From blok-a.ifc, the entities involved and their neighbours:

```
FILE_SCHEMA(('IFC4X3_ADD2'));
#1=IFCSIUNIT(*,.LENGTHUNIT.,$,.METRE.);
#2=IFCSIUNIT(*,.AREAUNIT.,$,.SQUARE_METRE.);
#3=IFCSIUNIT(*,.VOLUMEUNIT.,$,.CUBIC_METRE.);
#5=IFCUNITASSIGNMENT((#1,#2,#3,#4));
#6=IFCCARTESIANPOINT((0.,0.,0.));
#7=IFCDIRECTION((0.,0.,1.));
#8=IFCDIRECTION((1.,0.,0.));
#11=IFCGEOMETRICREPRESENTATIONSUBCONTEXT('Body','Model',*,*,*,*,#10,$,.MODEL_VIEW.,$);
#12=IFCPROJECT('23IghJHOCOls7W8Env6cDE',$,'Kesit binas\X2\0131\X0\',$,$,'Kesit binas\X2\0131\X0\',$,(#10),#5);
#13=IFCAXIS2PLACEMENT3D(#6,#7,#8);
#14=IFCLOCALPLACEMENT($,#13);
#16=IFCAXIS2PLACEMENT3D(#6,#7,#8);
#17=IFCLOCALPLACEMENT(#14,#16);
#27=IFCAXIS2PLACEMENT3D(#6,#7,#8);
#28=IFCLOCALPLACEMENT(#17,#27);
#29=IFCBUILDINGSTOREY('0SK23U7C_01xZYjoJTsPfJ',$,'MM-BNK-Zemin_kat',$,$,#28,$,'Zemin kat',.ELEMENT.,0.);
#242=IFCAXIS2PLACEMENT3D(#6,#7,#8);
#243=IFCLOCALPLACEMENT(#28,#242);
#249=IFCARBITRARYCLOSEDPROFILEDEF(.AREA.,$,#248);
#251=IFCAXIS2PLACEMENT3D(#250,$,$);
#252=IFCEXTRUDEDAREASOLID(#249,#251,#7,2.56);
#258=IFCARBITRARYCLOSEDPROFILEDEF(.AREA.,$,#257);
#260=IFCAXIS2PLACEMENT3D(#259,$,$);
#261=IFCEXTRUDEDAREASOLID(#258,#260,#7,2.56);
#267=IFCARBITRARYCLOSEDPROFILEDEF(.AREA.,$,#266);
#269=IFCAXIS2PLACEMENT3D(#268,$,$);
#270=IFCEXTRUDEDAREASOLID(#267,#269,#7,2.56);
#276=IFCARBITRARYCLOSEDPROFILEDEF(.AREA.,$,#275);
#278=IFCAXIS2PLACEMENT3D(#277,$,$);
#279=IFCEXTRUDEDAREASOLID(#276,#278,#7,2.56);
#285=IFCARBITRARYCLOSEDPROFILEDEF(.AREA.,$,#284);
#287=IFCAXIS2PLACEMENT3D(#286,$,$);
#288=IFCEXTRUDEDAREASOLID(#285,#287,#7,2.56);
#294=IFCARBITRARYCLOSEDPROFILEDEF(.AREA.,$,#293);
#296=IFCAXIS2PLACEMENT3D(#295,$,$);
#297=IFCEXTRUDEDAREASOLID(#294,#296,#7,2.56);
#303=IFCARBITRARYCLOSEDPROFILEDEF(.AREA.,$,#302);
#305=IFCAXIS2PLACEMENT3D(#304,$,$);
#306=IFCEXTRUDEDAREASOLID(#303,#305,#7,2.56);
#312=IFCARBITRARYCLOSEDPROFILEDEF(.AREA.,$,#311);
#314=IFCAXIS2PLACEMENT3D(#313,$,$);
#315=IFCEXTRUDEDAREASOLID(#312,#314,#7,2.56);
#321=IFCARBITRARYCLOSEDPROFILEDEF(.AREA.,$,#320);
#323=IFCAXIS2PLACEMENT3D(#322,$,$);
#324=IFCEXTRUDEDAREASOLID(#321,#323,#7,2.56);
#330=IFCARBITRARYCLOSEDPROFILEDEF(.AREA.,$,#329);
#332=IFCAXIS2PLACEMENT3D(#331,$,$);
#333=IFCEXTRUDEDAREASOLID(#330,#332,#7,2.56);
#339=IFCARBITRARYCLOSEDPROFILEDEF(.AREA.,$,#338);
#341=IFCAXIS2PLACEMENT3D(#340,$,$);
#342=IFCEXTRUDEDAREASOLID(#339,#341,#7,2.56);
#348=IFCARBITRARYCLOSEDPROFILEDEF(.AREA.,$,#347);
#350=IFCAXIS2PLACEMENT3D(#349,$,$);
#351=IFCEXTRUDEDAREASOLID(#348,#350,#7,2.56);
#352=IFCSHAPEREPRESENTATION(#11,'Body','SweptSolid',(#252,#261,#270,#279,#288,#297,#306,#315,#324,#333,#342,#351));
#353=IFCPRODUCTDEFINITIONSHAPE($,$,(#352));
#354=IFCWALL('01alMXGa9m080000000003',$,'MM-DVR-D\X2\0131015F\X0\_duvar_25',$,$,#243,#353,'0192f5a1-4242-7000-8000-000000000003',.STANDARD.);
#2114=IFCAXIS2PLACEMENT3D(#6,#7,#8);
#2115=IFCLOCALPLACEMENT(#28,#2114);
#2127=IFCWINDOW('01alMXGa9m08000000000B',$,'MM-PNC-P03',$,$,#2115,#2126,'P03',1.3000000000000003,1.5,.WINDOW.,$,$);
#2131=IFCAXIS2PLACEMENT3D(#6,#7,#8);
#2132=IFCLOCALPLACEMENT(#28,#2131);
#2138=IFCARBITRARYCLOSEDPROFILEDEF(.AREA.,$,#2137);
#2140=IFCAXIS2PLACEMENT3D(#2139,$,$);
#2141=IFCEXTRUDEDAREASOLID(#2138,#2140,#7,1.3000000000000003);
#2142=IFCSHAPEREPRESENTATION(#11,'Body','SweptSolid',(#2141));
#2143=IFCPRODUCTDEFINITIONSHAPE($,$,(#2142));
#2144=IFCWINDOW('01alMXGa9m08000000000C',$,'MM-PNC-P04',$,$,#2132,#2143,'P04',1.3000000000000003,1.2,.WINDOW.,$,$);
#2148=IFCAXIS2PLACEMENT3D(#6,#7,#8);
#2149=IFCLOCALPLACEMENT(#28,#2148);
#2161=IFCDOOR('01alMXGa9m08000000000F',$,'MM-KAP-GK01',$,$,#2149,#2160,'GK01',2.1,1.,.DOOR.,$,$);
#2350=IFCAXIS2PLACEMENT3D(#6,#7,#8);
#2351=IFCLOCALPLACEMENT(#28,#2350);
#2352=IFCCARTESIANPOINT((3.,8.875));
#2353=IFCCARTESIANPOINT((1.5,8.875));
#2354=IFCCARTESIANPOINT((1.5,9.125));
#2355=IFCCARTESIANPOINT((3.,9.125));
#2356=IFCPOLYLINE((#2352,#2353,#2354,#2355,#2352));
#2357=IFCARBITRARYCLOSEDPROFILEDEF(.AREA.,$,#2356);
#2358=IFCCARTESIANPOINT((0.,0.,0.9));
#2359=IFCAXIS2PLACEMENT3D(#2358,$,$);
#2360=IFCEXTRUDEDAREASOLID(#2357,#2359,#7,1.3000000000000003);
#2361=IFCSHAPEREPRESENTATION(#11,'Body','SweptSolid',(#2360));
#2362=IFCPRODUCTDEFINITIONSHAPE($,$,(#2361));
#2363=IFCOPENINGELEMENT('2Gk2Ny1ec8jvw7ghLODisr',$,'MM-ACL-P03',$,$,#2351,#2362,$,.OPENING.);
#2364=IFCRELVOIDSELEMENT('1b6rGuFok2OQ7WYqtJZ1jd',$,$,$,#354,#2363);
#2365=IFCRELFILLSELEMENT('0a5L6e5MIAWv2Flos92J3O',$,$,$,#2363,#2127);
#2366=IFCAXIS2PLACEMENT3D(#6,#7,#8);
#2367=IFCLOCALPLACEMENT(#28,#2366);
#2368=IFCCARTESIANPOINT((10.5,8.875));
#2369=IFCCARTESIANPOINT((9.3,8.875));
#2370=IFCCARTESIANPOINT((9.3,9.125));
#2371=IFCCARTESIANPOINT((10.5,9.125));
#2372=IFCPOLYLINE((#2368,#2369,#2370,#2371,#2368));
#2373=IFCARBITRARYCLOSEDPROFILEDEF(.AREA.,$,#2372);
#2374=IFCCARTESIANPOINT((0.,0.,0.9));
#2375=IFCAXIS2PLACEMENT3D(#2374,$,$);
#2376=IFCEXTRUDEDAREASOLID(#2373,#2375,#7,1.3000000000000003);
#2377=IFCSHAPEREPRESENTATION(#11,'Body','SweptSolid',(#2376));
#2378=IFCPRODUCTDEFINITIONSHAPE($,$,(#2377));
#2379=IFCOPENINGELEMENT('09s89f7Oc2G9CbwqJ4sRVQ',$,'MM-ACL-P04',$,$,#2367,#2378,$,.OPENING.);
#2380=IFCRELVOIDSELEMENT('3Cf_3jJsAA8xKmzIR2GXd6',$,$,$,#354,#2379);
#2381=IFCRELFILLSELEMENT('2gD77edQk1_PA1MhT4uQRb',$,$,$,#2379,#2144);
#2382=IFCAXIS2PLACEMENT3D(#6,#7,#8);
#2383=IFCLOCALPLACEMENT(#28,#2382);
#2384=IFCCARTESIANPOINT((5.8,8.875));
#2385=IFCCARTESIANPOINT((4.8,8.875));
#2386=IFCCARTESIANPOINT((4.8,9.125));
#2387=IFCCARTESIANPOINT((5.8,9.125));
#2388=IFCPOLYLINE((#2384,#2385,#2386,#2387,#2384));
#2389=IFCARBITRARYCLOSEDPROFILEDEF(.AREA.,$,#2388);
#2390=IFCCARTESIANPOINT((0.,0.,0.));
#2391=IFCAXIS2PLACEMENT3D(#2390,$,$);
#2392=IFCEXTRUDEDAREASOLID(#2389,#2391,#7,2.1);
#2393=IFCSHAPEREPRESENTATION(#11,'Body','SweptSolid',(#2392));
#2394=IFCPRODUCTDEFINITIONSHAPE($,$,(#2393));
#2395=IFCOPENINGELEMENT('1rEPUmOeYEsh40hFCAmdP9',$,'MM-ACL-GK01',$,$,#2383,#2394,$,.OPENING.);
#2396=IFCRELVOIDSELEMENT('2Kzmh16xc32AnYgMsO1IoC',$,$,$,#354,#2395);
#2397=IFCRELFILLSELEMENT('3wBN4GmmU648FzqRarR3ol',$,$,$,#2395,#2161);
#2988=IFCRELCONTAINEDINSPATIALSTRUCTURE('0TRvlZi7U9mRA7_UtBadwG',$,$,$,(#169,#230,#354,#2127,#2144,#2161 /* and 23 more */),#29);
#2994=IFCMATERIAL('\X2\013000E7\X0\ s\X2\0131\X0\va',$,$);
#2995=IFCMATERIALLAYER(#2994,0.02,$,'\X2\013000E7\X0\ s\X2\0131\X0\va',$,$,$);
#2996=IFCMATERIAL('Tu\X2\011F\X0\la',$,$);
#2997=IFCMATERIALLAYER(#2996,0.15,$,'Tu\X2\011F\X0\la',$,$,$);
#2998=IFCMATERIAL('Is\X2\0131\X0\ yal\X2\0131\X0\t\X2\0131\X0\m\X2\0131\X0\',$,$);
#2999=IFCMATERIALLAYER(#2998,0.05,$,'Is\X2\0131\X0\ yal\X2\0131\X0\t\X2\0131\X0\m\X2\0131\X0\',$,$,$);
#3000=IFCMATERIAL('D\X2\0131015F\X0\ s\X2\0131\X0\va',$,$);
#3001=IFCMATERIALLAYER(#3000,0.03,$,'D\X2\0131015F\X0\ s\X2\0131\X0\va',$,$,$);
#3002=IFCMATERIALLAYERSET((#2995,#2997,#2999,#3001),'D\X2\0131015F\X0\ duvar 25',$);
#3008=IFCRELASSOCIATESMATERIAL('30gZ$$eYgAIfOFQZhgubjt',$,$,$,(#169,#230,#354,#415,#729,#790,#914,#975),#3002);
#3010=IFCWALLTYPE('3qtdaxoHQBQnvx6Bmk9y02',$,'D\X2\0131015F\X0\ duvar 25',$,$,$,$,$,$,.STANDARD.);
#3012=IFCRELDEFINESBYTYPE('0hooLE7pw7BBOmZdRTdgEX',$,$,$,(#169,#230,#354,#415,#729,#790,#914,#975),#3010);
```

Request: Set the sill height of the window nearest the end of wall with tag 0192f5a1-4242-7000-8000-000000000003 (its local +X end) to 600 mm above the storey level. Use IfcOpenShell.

```python
import numpy as np
import ifcopenshell
import ifcopenshell.api.geometry
import ifcopenshell.geom
import ifcopenshell.util.element
import ifcopenshell.util.placement
import ifcopenshell.util.shape
import ifcopenshell.util.unit

model = ifcopenshell.open("blok-a.ifc")
unit_scale = ifcopenshell.util.unit.calculate_unit_scale(model)

window = model.by_guid("01alMXGa9m08000000000C")
opening = window.FillsVoids[0].RelatingOpeningElement
storey = ifcopenshell.util.element.get_container(window, ifc_class="IfcBuildingStorey")
level = ifcopenshell.util.placement.get_local_placement(storey.ObjectPlacement)[2, 3]

# The opening's origin need not be at the sill, so measure its lowest point.
shape = ifcopenshell.geom.create_shape(ifcopenshell.geom.settings(), opening)
bottom = ifcopenshell.util.shape.get_shape_bottom_elevation(shape, shape.geometry) / unit_scale
dz = level + 0.6 / unit_scale - bottom

shift = np.array([0.0, 0.0, dz])
# The window is not placed relative to its opening, so move both.
for product in (opening, window):
    matrix = ifcopenshell.util.placement.get_local_placement(product.ObjectPlacement)
    matrix[:3, 3] += shift
    ifcopenshell.api.geometry.edit_object_placement(model, product=product, matrix=matrix, is_si=False)

print(f"moved by {dz * unit_scale:+.3f} m")

model.write("blok-a_edited.ifc")
```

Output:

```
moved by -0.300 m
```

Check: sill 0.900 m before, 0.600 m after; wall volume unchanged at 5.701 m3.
